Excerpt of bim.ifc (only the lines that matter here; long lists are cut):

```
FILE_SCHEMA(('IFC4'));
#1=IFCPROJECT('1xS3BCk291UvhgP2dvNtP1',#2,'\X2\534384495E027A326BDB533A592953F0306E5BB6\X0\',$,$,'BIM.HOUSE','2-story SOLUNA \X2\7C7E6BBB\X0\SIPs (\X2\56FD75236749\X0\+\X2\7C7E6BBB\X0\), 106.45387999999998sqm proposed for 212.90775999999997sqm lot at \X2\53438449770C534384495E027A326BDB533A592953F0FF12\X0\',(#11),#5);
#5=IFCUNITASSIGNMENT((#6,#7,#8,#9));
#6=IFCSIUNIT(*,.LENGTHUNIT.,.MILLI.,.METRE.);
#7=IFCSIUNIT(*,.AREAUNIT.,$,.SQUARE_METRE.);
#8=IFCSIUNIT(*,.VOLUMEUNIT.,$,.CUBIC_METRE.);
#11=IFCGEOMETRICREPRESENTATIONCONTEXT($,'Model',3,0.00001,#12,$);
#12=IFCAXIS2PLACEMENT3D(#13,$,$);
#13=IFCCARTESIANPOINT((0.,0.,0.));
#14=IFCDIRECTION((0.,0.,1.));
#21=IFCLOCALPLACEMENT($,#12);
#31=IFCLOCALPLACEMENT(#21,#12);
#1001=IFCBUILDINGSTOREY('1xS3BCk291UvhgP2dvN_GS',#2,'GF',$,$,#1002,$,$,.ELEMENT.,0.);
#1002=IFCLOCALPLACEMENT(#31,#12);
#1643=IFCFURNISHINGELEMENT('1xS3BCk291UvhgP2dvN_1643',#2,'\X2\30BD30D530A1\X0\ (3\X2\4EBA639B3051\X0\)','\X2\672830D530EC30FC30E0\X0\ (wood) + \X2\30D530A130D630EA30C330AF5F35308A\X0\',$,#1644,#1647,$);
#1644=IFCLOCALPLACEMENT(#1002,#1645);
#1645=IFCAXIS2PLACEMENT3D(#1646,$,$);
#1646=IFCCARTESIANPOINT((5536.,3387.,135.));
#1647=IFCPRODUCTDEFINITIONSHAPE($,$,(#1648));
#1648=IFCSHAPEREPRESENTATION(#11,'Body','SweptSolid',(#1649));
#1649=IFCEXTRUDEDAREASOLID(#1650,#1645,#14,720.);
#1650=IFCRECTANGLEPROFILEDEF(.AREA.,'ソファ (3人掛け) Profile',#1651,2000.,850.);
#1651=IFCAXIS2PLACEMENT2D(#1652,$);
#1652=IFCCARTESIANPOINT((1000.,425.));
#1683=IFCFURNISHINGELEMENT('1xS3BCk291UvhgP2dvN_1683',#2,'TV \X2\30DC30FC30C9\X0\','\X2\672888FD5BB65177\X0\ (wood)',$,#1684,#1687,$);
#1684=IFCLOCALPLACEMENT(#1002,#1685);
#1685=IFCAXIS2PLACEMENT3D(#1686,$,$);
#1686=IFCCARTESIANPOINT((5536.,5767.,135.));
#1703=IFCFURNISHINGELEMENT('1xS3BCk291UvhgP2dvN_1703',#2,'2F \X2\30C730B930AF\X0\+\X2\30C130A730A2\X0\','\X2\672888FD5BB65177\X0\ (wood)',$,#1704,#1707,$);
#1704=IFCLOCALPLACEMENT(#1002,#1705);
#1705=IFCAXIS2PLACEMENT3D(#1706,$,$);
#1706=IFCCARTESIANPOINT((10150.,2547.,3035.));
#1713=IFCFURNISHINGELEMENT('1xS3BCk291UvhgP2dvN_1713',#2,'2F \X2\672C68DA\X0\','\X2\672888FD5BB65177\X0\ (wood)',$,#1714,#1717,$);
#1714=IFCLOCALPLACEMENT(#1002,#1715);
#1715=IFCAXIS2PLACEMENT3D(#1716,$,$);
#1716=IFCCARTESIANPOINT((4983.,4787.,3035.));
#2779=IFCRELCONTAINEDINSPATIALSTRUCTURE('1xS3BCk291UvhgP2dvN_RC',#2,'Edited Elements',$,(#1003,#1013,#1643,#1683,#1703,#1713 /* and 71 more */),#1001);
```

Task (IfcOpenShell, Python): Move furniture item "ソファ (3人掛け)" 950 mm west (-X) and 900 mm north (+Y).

```python
import ifcopenshell
import ifcopenshell.api.geometry
import ifcopenshell.util.placement
import ifcopenshell.util.unit

model = ifcopenshell.open("bim.ifc")
unit_scale = ifcopenshell.util.unit.calculate_unit_scale(model)

item = model.by_guid("1xS3BCk291UvhgP2dvN_1643")
matrix = ifcopenshell.util.placement.get_local_placement(item.ObjectPlacement)
matrix[0, 3] -= 0.95 / unit_scale
matrix[1, 3] += 0.9 / unit_scale
ifcopenshell.api.geometry.edit_object_placement(model, product=item, matrix=matrix, is_si=False)

print(ifcopenshell.util.placement.get_local_placement(item.ObjectPlacement).round(3) + 0.0)

model.write("bim_rev.ifc")
```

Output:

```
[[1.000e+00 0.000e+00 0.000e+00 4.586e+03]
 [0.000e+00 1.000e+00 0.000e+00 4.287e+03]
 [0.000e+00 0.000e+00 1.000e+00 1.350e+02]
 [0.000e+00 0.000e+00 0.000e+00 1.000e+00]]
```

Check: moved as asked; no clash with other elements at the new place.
